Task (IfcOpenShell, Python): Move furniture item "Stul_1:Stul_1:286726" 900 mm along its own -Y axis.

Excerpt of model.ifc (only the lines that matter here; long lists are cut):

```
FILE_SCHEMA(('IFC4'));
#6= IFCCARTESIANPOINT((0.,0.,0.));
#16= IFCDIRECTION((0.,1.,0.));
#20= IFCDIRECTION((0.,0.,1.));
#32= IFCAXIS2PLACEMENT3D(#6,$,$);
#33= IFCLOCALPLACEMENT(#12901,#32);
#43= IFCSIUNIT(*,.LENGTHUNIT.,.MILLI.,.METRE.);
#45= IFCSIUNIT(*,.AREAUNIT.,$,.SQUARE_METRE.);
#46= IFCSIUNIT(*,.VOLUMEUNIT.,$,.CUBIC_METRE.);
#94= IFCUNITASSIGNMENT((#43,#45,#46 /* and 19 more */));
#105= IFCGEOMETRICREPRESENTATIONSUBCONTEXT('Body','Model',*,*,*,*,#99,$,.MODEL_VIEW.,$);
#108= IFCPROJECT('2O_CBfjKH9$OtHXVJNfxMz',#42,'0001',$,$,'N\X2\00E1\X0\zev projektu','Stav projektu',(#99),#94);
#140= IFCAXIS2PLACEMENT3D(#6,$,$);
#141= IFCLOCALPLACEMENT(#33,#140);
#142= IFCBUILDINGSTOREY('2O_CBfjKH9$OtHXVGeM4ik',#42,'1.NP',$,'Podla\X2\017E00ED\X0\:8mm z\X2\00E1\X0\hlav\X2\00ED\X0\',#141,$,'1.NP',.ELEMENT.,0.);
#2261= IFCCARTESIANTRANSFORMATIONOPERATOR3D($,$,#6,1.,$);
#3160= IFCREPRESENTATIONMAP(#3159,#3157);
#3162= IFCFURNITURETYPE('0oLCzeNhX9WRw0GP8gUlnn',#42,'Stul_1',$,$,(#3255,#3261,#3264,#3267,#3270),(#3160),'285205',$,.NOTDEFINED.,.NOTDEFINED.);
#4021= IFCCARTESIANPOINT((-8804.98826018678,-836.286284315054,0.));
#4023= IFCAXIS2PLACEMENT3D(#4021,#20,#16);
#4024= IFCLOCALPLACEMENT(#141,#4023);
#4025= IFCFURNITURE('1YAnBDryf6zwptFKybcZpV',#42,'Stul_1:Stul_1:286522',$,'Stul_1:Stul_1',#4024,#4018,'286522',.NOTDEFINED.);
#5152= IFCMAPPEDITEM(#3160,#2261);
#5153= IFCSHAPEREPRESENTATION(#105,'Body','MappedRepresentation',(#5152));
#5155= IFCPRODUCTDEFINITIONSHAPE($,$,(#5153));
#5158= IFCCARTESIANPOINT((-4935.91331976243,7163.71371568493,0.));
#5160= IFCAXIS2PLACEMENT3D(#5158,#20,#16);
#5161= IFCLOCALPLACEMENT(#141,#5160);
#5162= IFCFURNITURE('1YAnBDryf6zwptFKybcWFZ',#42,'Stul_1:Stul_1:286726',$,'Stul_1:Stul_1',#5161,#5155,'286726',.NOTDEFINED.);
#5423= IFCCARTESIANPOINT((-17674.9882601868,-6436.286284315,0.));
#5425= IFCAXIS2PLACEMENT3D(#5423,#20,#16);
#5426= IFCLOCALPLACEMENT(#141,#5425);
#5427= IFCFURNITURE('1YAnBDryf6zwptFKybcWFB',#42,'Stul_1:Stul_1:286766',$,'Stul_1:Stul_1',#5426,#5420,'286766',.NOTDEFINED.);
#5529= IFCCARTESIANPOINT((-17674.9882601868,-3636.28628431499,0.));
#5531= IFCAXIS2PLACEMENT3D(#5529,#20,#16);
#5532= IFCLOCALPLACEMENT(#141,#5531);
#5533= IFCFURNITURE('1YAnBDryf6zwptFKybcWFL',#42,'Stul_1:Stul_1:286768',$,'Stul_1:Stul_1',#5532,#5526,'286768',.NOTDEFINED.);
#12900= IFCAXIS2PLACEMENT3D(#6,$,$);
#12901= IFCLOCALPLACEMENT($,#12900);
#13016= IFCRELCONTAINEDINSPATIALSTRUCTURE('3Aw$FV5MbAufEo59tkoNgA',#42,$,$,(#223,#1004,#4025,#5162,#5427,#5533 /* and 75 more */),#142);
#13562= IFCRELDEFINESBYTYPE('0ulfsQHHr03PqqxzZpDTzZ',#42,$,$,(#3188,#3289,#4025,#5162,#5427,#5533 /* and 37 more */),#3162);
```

```python
import ifcopenshell
import ifcopenshell.api.geometry
import ifcopenshell.util.placement
import ifcopenshell.util.unit

model = ifcopenshell.open("model.ifc")
unit_scale = ifcopenshell.util.unit.calculate_unit_scale(model)

item = model.by_id(5162)
matrix = ifcopenshell.util.placement.get_local_placement(item.ObjectPlacement)
matrix[:3, 3] -= matrix[:3, 1] * 0.9 / unit_scale
ifcopenshell.api.geometry.edit_object_placement(model, product=item, matrix=matrix, is_si=False)

print(ifcopenshell.util.placement.get_local_placement(item.ObjectPlacement).round(3) + 0.0)

model.write("model_edited.ifc")
```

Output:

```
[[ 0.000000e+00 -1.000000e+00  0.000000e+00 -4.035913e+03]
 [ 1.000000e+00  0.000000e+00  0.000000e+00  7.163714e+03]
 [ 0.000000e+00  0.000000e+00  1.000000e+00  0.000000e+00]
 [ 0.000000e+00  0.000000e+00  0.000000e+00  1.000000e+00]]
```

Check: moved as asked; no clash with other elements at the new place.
